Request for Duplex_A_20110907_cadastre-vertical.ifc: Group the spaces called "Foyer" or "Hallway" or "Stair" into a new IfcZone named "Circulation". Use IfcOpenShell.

First a look at what the model holds.

```python
import ifcopenshell

model = ifcopenshell.open("Duplex_A_20110907_cadastre-vertical.ifc")
print(model.schema)
seen = {}
for space in model.by_type("IfcSpace"):
    seen[space.LongName] = seen.get(space.LongName, 0) + 1
for name, count in sorted(seen.items(), key=str):
    print(count, "x", name)
print("zones:", [z.Name for z in model.by_type("IfcZone")][:20])
```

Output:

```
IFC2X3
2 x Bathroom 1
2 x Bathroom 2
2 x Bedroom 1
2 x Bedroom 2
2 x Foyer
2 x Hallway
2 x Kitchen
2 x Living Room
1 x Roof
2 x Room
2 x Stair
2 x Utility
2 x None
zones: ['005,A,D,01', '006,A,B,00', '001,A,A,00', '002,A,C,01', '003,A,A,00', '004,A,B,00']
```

```python
import ifcopenshell
import ifcopenshell.api.group
import ifcopenshell.api.root

model = ifcopenshell.open("Duplex_A_20110907_cadastre-vertical.ifc")

names = {"Foyer", "Hallway", "Stair"}
spaces = [s for s in model.by_type("IfcSpace") if s.LongName in names]

zone = ifcopenshell.api.root.create_entity(model, ifc_class="IfcZone", name="Circulation")
ifcopenshell.api.group.assign_group(model, products=spaces, group=zone)
print(len(spaces), "spaces in", zone.Name)

model.write("Duplex_A_20110907_cadastre-vertical-out.ifc")
```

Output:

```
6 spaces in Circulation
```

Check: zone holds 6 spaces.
